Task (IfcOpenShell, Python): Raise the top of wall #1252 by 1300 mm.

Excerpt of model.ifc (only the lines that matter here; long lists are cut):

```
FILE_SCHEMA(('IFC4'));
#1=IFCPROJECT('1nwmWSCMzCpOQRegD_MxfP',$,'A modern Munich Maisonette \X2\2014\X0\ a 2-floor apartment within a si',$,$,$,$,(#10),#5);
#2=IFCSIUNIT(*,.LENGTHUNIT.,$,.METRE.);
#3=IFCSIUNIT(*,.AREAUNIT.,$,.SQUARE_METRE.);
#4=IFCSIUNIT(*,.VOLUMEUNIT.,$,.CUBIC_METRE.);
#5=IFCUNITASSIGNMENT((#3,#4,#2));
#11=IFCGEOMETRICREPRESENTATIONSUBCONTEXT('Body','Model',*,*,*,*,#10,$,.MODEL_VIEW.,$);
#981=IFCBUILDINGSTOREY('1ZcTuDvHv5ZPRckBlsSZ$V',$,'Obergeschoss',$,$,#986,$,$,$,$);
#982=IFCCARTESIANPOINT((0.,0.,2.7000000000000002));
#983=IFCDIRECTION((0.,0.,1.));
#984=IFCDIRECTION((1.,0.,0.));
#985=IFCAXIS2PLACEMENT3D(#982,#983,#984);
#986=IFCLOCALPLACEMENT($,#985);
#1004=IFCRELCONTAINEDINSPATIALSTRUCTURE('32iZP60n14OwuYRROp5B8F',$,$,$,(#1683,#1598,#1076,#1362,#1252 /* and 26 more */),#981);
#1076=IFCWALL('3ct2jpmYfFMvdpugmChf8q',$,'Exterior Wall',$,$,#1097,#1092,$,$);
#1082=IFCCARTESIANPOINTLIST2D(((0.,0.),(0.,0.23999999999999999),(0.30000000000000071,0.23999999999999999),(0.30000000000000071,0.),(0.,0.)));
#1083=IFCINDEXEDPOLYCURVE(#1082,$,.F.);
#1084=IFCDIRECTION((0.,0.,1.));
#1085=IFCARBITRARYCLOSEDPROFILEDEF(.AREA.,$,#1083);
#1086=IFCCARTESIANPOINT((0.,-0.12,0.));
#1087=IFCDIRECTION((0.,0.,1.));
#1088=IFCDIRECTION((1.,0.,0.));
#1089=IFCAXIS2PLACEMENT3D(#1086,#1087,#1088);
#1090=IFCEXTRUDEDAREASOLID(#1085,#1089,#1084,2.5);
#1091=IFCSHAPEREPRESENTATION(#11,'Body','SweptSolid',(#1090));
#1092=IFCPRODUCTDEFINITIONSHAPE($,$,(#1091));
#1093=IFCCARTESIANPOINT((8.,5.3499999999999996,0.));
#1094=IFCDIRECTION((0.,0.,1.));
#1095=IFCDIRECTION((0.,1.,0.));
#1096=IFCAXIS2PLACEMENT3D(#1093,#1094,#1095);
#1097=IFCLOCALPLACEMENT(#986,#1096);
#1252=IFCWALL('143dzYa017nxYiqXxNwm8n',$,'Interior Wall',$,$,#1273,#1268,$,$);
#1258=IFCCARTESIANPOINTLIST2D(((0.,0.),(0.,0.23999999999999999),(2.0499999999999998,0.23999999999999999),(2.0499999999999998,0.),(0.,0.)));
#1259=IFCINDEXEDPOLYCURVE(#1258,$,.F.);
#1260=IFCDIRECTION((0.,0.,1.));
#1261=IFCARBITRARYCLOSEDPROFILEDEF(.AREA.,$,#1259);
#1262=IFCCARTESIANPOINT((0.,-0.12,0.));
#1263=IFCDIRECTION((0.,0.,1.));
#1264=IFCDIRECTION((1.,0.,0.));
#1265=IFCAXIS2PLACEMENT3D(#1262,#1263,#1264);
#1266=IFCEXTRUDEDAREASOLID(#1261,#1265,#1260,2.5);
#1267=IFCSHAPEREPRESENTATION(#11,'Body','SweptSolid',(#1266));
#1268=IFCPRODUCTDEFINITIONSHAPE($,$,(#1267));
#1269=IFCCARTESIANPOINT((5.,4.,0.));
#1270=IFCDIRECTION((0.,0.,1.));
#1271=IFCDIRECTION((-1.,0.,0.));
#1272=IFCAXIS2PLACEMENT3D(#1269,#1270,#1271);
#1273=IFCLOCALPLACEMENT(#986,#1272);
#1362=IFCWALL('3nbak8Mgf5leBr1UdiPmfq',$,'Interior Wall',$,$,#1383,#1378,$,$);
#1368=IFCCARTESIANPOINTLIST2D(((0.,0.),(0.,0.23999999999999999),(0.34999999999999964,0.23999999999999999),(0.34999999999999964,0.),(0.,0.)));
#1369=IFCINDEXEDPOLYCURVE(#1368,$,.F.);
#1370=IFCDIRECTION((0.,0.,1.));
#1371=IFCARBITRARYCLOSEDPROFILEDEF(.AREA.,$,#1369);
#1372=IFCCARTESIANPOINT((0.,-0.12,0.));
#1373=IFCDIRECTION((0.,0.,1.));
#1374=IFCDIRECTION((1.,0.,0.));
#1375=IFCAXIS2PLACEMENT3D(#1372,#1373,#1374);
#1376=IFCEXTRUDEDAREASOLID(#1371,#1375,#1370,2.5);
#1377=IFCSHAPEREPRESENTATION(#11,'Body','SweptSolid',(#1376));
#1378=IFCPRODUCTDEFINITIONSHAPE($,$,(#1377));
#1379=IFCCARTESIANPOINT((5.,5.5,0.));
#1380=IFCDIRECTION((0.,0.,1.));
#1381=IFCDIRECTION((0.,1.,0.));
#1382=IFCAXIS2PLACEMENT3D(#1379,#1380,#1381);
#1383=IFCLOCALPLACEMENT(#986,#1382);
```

```python
import ifcopenshell
import ifcopenshell.geom
import ifcopenshell.util.representation
import ifcopenshell.util.shape
import ifcopenshell.util.unit

model = ifcopenshell.open("model.ifc")
unit_scale = ifcopenshell.util.unit.calculate_unit_scale(model)
settings = ifcopenshell.geom.settings()


def volume(element):
    """Net volume in cubic metres, openings subtracted."""
    shape = ifcopenshell.geom.create_shape(settings, element)
    return ifcopenshell.util.shape.get_volume(shape.geometry)


wall = model.by_guid("143dzYa017nxYiqXxNwm8n")
before = volume(wall)

body = ifcopenshell.util.representation.get_representation(wall, "Model", "Body")
solid = body.Items[0]
old_height = solid.Depth
solid.Depth += 1.3 / unit_scale
after = volume(wall)

print(f"height {old_height:g} -> {solid.Depth:g}, volume {before:.3f} -> {after:.3f} m3")

model.write("model_updated.ifc")
```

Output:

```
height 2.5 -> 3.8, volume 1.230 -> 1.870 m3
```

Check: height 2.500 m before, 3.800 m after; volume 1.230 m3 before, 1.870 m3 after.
